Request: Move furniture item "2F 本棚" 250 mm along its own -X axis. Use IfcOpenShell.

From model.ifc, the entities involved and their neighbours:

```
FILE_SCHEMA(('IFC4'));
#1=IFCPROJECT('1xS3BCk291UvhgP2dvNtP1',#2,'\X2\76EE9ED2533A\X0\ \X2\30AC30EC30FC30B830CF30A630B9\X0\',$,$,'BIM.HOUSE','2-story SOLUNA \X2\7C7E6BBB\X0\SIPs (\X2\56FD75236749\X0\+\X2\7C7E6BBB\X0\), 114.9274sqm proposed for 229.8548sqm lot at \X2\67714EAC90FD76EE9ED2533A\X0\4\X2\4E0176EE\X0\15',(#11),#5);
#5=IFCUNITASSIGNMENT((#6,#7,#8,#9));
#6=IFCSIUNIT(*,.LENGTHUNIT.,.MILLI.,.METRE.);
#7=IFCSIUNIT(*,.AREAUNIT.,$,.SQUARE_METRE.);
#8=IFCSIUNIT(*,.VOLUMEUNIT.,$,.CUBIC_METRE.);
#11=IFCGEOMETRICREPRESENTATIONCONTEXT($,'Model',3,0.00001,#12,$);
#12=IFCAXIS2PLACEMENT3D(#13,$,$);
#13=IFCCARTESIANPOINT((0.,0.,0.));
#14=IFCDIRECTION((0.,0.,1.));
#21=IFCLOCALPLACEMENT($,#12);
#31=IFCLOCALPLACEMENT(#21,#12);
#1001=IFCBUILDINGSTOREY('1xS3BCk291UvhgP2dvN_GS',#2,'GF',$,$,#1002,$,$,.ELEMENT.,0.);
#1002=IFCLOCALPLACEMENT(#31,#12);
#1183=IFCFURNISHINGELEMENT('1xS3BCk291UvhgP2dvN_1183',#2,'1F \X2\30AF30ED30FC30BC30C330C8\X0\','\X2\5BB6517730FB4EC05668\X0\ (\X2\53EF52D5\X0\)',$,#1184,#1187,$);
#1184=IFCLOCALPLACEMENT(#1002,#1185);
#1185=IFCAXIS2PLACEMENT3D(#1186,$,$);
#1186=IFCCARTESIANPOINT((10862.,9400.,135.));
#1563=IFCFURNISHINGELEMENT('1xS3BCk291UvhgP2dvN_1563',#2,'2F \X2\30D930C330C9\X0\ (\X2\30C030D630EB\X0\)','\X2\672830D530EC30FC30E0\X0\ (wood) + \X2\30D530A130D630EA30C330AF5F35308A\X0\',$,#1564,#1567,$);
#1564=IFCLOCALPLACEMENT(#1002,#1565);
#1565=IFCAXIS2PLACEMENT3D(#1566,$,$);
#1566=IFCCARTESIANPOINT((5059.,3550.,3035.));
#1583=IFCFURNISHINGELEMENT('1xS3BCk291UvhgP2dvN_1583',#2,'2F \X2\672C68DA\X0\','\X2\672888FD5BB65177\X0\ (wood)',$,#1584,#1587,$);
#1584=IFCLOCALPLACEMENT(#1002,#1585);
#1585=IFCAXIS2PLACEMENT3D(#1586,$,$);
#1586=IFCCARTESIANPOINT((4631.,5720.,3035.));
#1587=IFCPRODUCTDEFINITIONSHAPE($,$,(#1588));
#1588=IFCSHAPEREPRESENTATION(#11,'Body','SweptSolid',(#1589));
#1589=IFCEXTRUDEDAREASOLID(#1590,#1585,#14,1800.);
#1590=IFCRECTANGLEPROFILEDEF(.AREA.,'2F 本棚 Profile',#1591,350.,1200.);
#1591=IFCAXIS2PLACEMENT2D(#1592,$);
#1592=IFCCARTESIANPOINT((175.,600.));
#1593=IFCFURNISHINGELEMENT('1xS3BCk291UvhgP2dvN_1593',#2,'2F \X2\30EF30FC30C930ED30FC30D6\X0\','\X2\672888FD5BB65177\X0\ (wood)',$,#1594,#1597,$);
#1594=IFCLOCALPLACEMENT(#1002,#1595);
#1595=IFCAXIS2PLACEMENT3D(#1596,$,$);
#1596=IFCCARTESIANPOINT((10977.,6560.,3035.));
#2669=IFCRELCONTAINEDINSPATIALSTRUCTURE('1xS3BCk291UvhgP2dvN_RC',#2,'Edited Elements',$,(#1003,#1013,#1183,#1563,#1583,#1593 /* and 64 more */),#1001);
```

```python
import ifcopenshell
import ifcopenshell.api.geometry
import ifcopenshell.util.placement

model = ifcopenshell.open("model.ifc")

item = model.by_guid("1xS3BCk291UvhgP2dvN_1583")
matrix = ifcopenshell.util.placement.get_local_placement(item.ObjectPlacement)
matrix[:3, 3] -= matrix[:3, 0] * 250.0
ifcopenshell.api.geometry.edit_object_placement(model, product=item, matrix=matrix, is_si=False)

print(ifcopenshell.util.placement.get_local_placement(item.ObjectPlacement).round(3) + 0.0)

model.write("model_rev.ifc")
```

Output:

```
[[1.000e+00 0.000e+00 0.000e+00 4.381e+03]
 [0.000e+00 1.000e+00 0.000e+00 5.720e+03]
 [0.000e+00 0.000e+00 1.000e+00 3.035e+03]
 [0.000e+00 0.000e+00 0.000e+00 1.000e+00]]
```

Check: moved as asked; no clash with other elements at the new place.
